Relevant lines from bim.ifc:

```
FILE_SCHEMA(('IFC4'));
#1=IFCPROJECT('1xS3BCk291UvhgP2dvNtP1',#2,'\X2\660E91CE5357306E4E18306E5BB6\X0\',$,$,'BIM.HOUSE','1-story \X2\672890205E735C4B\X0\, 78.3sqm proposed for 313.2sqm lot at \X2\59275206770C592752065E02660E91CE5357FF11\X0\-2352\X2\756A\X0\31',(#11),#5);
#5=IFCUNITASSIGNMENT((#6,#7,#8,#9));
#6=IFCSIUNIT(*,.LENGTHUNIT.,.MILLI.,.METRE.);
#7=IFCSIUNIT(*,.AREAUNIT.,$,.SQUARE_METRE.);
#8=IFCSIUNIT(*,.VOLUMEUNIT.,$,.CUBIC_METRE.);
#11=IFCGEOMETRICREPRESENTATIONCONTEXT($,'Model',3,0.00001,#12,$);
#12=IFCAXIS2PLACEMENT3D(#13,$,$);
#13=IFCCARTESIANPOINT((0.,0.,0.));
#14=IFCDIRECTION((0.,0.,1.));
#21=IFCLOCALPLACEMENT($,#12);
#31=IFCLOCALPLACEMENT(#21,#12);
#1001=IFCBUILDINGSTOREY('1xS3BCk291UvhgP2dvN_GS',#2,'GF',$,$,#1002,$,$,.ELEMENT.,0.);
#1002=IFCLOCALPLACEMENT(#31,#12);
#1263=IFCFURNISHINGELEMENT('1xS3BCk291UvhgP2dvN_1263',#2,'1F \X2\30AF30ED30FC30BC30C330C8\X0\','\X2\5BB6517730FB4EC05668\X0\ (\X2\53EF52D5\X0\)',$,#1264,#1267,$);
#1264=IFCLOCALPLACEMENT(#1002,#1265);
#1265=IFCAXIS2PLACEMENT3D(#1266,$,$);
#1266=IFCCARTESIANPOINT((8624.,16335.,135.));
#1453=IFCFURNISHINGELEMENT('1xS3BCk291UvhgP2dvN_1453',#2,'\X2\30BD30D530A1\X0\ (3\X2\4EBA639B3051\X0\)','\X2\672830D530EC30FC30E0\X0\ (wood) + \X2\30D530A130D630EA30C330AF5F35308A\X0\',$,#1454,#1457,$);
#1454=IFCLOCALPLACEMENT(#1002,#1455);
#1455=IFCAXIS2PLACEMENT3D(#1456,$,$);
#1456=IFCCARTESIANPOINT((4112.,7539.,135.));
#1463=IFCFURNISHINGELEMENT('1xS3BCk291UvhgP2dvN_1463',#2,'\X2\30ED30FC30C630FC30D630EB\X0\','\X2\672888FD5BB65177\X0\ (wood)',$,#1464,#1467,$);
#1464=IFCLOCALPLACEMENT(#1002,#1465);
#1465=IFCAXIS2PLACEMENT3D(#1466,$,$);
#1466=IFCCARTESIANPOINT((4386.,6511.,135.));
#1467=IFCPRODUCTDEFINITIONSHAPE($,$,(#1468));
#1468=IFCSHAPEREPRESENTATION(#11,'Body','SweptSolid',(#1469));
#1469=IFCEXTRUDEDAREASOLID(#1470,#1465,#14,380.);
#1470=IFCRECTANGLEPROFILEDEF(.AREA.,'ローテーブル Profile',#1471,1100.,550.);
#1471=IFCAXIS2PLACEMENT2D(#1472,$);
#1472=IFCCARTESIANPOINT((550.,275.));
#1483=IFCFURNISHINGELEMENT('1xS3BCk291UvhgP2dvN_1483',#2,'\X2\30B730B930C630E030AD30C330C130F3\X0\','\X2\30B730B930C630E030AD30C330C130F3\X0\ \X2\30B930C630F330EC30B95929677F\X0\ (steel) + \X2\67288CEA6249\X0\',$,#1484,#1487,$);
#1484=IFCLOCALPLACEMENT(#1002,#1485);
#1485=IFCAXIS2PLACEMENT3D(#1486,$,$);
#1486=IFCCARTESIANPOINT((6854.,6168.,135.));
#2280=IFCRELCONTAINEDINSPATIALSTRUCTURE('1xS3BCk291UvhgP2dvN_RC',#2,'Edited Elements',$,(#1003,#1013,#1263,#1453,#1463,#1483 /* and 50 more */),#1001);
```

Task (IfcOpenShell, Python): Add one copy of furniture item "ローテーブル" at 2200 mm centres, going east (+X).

```python
import numpy as np
import ifcopenshell
import ifcopenshell.api.geometry
import ifcopenshell.api.root
import ifcopenshell.util.element
import ifcopenshell.util.placement
import ifcopenshell.util.unit

model = ifcopenshell.open("bim.ifc")
unit_scale = ifcopenshell.util.unit.calculate_unit_scale(model)


def reuse_history(source, copy):
    """copy_class also copies each property set's owner history, people and application; keep the originals."""
    for rel in copy.IsDefinedBy:
        if rel.is_a("IfcRelDefinesByProperties") and (history := rel.RelatingPropertyDefinition.OwnerHistory):
            rel.RelatingPropertyDefinition.OwnerHistory = source.OwnerHistory
            ifcopenshell.util.element.remove_deep2(model, history)


source = model.by_guid("1xS3BCk291UvhgP2dvN_1463")
base = ifcopenshell.util.placement.get_local_placement(source.ObjectPlacement)
step = np.array([1.0, 0.0, 0.0]) * 2.2 / unit_scale

for i in range(1, 2):
    copy = ifcopenshell.api.root.copy_class(model, product=source)
    copy.Representation = ifcopenshell.util.element.copy_deep(
        model, source.Representation, exclude=["IfcGeometricRepresentationContext", "IfcRepresentationMap"]
    )
    reuse_history(source, copy)
    matrix = base.copy()
    matrix[:3, 3] += i * step
    print("added at", matrix[:3, 3].round(3) + 0.0)
    ifcopenshell.api.geometry.edit_object_placement(model, product=copy, matrix=matrix, is_si=False)

model.write("bim_updated.ifc")
```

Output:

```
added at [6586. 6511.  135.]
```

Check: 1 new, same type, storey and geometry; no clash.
